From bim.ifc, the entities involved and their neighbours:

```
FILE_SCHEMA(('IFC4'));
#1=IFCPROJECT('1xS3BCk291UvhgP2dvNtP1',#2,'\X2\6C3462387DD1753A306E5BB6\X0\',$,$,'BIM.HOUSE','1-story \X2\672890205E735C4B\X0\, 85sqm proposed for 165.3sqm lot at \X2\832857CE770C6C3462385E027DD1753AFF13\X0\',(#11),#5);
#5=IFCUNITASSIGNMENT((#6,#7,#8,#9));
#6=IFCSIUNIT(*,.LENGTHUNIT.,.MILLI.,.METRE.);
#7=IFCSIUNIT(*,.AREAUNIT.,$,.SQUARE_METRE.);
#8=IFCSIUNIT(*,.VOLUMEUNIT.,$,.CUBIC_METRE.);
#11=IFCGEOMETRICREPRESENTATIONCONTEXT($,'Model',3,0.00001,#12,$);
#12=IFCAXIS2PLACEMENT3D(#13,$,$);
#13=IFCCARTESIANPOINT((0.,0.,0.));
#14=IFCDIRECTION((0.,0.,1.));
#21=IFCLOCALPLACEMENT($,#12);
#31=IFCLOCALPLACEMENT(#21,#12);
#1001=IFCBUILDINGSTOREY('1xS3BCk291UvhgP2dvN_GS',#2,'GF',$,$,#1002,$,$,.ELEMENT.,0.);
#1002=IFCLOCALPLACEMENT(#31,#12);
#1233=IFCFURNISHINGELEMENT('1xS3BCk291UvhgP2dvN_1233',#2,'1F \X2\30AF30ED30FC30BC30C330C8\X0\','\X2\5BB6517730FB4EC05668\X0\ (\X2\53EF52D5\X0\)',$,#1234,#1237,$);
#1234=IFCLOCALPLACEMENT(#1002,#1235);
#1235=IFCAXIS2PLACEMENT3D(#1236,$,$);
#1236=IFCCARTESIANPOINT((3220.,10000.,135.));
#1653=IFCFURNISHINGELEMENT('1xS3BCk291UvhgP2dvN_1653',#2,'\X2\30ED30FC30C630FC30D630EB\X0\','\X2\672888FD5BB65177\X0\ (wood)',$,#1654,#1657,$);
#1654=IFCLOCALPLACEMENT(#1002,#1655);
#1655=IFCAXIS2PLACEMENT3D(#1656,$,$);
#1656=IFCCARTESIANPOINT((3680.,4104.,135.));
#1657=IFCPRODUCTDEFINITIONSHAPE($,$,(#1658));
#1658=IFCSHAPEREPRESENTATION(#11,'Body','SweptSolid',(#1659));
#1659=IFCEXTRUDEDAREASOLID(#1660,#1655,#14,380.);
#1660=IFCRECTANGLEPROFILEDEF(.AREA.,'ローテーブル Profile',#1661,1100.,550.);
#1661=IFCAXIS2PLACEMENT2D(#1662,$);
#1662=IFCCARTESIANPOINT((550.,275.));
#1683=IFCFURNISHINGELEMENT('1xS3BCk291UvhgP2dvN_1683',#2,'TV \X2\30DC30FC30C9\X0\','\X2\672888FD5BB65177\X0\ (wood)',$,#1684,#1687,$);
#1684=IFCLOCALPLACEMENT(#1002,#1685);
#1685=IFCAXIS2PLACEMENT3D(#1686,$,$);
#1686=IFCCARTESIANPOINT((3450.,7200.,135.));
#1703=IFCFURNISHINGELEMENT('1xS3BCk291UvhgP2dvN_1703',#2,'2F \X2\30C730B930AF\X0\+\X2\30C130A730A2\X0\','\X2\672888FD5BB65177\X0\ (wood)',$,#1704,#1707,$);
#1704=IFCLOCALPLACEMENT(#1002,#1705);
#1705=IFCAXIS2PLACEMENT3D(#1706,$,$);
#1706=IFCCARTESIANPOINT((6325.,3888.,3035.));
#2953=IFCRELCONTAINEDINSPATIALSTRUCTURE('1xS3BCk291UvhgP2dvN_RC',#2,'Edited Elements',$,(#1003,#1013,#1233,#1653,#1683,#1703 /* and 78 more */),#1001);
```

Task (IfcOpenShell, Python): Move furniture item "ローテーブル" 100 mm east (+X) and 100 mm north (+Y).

```python
import ifcopenshell
import ifcopenshell.api.geometry
import ifcopenshell.util.placement
import ifcopenshell.util.unit

model = ifcopenshell.open("bim.ifc")
unit_scale = ifcopenshell.util.unit.calculate_unit_scale(model)

item = model.by_guid("1xS3BCk291UvhgP2dvN_1653")
matrix = ifcopenshell.util.placement.get_local_placement(item.ObjectPlacement)
matrix[0, 3] += 0.1 / unit_scale
matrix[1, 3] += 0.1 / unit_scale
ifcopenshell.api.geometry.edit_object_placement(model, product=item, matrix=matrix, is_si=False)

print(ifcopenshell.util.placement.get_local_placement(item.ObjectPlacement).round(3) + 0.0)

model.write("bim_edited.ifc")
```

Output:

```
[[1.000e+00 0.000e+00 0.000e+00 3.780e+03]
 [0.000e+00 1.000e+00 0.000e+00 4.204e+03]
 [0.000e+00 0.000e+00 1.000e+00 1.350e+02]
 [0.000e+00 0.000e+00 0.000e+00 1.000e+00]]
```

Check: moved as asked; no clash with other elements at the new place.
